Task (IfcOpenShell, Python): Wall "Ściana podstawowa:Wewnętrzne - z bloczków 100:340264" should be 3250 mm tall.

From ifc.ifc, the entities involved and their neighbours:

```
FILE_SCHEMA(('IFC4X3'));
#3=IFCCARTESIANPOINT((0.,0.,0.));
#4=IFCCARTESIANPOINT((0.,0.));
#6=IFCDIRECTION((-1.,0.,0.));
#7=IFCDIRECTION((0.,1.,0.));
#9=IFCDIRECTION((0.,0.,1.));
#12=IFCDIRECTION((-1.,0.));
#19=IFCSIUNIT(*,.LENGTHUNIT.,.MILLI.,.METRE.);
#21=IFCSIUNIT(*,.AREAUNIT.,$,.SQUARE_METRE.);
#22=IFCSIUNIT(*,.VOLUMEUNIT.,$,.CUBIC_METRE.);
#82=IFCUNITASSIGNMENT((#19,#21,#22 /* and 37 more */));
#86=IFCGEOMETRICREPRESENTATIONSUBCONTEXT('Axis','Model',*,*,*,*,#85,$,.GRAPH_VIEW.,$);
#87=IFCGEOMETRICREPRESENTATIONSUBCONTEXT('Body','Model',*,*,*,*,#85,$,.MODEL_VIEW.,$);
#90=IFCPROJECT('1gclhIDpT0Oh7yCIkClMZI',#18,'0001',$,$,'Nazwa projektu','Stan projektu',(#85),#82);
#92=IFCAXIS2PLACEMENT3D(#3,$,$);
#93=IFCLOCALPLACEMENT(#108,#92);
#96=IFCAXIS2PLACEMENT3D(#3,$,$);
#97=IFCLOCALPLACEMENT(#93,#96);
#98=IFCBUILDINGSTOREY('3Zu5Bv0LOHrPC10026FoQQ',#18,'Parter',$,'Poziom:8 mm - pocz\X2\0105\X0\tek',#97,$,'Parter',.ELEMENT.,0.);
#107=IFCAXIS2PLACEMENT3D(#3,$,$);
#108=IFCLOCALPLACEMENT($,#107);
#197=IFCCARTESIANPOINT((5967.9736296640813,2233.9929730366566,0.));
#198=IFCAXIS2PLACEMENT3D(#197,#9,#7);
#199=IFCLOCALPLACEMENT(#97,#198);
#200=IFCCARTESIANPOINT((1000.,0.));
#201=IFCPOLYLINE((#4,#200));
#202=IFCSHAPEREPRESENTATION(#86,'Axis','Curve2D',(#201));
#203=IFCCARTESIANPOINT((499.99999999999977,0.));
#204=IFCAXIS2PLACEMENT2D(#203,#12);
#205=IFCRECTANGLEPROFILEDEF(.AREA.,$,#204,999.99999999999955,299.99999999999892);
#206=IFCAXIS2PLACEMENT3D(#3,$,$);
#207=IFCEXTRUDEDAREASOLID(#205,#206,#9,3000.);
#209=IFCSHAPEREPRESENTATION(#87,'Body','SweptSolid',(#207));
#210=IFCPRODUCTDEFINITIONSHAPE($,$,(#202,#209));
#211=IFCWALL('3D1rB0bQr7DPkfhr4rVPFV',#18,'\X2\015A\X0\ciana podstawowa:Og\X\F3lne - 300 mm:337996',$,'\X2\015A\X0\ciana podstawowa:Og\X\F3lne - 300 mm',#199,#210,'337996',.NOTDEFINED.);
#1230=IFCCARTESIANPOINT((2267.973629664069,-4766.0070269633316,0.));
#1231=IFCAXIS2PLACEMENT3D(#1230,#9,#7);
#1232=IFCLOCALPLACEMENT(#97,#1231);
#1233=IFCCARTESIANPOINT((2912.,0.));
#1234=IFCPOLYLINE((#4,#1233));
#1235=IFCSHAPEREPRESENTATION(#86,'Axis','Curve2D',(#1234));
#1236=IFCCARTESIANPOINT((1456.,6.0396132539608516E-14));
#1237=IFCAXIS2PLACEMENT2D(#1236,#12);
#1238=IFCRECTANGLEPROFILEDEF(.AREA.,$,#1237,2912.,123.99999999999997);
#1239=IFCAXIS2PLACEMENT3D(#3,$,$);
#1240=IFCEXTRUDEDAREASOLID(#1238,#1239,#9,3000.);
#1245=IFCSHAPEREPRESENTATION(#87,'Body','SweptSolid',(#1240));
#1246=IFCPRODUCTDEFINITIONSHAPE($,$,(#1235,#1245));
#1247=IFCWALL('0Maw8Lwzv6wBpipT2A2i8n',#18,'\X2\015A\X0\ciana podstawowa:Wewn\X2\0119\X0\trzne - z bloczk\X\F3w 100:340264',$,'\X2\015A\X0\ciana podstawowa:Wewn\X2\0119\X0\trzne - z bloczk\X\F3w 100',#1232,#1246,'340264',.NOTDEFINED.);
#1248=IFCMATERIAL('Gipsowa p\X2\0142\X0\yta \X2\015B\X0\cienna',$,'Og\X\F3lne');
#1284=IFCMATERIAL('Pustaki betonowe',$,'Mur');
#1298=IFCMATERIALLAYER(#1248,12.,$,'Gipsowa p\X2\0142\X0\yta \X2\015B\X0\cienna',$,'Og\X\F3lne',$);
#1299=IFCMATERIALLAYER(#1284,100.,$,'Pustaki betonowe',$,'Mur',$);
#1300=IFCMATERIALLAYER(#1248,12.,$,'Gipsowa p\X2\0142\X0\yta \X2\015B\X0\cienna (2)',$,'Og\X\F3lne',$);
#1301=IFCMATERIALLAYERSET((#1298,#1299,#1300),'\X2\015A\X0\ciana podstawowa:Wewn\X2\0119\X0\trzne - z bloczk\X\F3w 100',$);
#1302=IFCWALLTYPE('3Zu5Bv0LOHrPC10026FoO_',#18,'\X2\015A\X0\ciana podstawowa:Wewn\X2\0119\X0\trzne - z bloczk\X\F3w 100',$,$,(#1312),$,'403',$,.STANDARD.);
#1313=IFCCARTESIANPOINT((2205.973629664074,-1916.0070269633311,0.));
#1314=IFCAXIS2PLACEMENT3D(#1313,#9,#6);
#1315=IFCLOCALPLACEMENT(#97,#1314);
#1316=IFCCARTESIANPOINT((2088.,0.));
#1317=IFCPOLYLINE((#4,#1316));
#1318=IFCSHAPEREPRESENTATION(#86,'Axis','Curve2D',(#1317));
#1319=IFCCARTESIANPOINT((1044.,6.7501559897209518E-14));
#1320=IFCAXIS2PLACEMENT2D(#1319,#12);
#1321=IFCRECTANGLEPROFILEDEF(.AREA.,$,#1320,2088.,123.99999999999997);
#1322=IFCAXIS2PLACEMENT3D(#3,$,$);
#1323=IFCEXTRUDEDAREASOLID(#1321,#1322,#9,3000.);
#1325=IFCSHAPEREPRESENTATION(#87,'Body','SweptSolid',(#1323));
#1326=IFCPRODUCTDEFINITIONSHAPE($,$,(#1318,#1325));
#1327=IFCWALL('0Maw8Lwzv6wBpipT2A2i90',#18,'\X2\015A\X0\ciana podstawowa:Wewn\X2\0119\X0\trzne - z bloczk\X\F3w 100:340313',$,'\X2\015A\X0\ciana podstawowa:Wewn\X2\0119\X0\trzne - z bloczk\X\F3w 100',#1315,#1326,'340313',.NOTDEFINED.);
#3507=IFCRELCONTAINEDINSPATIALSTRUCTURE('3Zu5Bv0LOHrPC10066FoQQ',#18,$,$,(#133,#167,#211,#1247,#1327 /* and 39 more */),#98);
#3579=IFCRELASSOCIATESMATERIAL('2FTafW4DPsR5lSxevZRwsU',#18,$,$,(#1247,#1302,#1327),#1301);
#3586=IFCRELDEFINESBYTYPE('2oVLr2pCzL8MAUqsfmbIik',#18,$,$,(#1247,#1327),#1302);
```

```python
import ifcopenshell
import ifcopenshell.geom
import ifcopenshell.util.representation
import ifcopenshell.util.shape

model = ifcopenshell.open("ifc.ifc")
settings = ifcopenshell.geom.settings()


def volume(element):
    """Net volume in cubic metres, openings subtracted."""
    shape = ifcopenshell.geom.create_shape(settings, element)
    return ifcopenshell.util.shape.get_volume(shape.geometry)


wall = model.by_id(1247)
before = volume(wall)

body = ifcopenshell.util.representation.get_representation(wall, "Model", "Body")
solid = body.Items[0]
old_height = solid.Depth
solid.Depth = 3250.0
after = volume(wall)

print(f"height {old_height:g} -> {solid.Depth:g}, volume {before:.3f} -> {after:.3f} m3")

model.write("ifc_rev.ifc")
```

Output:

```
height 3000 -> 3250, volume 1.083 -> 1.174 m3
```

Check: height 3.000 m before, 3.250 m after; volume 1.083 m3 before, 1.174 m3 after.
